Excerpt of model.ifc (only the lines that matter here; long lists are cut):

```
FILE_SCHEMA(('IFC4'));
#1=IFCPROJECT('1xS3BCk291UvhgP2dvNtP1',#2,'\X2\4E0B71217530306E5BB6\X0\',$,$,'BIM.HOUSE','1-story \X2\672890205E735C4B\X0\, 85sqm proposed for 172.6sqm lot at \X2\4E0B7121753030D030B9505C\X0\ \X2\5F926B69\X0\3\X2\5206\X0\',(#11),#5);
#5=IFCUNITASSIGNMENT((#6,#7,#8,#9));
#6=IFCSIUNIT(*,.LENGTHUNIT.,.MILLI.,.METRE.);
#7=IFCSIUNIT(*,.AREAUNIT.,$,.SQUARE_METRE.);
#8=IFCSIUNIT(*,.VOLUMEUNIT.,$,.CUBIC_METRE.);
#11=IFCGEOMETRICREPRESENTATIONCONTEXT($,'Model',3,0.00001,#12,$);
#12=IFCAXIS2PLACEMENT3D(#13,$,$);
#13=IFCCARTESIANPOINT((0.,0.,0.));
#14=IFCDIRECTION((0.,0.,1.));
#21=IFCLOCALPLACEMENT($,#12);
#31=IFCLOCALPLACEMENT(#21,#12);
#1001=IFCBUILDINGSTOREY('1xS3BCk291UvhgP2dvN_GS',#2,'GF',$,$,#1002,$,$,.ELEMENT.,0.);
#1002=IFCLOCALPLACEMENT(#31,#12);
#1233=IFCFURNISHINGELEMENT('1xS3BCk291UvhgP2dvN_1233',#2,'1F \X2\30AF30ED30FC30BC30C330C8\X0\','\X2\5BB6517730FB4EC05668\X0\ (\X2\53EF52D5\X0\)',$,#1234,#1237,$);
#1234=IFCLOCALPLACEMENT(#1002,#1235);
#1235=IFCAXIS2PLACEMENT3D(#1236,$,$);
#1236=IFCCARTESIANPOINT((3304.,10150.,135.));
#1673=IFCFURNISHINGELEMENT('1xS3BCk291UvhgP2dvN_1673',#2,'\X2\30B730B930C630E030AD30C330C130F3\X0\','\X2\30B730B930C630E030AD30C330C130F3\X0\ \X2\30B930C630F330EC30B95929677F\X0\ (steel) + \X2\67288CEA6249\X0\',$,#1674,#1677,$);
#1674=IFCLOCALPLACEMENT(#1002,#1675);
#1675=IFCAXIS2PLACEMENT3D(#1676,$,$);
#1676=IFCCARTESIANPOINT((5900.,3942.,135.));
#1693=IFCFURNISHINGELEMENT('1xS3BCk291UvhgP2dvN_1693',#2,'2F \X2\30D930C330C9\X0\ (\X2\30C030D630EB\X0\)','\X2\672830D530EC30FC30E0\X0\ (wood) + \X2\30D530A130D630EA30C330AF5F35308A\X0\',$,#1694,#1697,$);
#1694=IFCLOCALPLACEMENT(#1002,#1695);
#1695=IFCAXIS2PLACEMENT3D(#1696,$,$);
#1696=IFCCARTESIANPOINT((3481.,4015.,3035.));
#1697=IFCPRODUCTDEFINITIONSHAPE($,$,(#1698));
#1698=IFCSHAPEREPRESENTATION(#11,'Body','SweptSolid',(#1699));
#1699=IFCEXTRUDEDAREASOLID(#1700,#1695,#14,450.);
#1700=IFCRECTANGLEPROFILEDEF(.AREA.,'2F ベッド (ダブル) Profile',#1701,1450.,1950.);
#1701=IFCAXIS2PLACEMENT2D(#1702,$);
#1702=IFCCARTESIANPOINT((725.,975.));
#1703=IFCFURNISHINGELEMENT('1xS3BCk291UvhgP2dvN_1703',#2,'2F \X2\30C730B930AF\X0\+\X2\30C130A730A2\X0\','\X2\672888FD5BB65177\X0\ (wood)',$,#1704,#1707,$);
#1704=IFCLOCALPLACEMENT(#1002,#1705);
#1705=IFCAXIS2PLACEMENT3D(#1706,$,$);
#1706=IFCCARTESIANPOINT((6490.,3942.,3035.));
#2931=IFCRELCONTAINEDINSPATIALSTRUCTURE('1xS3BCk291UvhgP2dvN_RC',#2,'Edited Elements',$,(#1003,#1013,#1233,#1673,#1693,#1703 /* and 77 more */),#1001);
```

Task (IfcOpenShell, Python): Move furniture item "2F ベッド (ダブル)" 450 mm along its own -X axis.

```python
import ifcopenshell
import ifcopenshell.api.geometry
import ifcopenshell.util.placement
import ifcopenshell.util.unit

model = ifcopenshell.open("model.ifc")
unit_scale = ifcopenshell.util.unit.calculate_unit_scale(model)

item = model.by_id(1693)
matrix = ifcopenshell.util.placement.get_local_placement(item.ObjectPlacement)
matrix[:3, 3] -= matrix[:3, 0] * 0.45 / unit_scale
ifcopenshell.api.geometry.edit_object_placement(model, product=item, matrix=matrix, is_si=False)

print(ifcopenshell.util.placement.get_local_placement(item.ObjectPlacement).round(3) + 0.0)

model.write("model_edited.ifc")
```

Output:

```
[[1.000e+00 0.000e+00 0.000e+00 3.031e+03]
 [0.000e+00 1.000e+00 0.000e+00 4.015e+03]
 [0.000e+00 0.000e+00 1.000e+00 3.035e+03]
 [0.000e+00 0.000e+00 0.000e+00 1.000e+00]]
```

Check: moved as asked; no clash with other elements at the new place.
